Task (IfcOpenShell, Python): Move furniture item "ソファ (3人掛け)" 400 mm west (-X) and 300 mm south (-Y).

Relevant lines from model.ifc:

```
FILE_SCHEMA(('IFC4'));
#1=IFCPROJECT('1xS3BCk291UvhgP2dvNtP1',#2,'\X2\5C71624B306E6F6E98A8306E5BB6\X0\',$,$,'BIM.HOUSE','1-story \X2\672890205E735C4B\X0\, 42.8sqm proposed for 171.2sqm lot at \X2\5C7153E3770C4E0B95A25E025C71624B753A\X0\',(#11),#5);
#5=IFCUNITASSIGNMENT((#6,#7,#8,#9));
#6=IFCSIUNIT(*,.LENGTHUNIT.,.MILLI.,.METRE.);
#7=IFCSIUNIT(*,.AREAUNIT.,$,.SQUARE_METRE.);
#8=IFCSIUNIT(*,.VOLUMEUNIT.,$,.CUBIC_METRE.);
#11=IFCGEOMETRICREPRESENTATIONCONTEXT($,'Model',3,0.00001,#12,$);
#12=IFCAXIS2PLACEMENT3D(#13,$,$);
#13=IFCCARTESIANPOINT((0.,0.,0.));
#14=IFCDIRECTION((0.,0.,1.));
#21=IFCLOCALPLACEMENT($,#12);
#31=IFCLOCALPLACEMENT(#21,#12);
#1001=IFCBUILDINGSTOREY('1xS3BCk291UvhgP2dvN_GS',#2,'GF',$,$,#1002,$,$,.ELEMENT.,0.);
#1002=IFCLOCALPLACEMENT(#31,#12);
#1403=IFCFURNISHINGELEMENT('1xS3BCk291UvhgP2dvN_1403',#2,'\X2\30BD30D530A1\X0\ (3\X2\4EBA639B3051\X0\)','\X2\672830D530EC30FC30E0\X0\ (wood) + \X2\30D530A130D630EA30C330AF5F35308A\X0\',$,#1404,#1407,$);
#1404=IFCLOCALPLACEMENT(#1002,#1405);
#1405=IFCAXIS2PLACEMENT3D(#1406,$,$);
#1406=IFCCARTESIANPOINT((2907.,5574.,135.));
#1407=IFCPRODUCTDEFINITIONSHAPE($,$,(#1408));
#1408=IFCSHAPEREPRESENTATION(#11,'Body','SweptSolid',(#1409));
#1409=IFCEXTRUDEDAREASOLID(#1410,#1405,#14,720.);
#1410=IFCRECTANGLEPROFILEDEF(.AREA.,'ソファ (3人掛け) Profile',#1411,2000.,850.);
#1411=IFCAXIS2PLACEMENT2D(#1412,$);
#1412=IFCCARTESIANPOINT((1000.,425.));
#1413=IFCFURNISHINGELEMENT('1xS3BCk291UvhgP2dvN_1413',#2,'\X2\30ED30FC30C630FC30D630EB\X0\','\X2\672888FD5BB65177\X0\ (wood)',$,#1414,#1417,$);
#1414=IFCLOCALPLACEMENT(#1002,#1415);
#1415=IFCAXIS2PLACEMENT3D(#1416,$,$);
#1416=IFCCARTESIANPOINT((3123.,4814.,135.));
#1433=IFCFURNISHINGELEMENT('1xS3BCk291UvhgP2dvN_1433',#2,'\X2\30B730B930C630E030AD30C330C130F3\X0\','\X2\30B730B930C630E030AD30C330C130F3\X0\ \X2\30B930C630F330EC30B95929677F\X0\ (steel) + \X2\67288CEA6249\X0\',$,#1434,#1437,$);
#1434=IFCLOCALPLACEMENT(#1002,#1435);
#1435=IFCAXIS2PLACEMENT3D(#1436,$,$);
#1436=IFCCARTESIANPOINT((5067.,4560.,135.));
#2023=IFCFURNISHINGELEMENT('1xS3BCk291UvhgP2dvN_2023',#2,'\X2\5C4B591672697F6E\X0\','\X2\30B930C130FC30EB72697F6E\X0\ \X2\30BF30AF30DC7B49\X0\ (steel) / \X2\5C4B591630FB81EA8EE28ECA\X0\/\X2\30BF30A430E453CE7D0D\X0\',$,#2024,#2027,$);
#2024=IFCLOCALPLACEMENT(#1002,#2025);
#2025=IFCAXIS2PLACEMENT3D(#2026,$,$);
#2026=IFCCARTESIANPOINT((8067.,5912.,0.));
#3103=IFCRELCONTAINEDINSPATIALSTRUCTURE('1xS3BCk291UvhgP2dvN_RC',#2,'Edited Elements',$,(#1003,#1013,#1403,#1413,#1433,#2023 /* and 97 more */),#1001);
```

```python
import ifcopenshell
import ifcopenshell.api.geometry
import ifcopenshell.util.placement

model = ifcopenshell.open("model.ifc")

item = model.by_id(1403)
matrix = ifcopenshell.util.placement.get_local_placement(item.ObjectPlacement)
matrix[0, 3] -= 400.0
matrix[1, 3] -= 300.0
ifcopenshell.api.geometry.edit_object_placement(model, product=item, matrix=matrix, is_si=False)

print(ifcopenshell.util.placement.get_local_placement(item.ObjectPlacement).round(3) + 0.0)

model.write("model-out.ifc")
```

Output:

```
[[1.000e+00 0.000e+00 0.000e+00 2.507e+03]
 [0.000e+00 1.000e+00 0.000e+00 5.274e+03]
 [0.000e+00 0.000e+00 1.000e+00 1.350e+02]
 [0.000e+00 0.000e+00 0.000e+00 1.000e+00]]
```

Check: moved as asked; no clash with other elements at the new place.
